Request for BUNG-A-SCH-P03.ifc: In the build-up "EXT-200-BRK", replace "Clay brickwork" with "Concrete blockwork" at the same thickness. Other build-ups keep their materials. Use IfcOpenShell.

First a look at what the model holds.

```python
import ifcopenshell
import ifcopenshell.util.element

model = ifcopenshell.open("BUNG-A-SCH-P03.ifc")
print(model.schema)
for layer_set in model.by_type("IfcMaterialLayerSet"):
    if layer_set.LayerSetName == "EXT-200-BRK":
        for layer in layer_set.MaterialLayers:
            print(layer.id(), layer.Material and layer.Material.Name, layer.LayerThickness, sep=" | ")
        print(len(ifcopenshell.util.element.get_elements_by_material(model, layer_set)), "elements and types use it")
print(sorted(m.Name for m in model.by_type("IfcMaterial") if m.Name)[:60])
```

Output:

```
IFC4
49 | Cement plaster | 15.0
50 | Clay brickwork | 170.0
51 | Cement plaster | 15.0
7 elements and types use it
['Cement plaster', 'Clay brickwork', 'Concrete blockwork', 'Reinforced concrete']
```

```python
import ifcopenshell
import ifcopenshell.api.material

model = ifcopenshell.open("BUNG-A-SCH-P03.ifc")

layer_set = next(s for s in model.by_type("IfcMaterialLayerSet") if s.LayerSetName == "EXT-200-BRK")
layer = next(l for l in layer_set.MaterialLayers if l.Material and l.Material.Name == "Clay brickwork")
material = next(m for m in model.by_type("IfcMaterial") if m.Name == "Concrete blockwork")

# Point this one layer at the other material; renaming the old one would change it everywhere.
ifcopenshell.api.material.edit_layer(model, layer=layer, attributes={"Name": material.Name}, material=material)

print([l.Material.Name if l.Material else None for l in layer_set.MaterialLayers])

model.write("BUNG-A-SCH-P03_updated.ifc")
```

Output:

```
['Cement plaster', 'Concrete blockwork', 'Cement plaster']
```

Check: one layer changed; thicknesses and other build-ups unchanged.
